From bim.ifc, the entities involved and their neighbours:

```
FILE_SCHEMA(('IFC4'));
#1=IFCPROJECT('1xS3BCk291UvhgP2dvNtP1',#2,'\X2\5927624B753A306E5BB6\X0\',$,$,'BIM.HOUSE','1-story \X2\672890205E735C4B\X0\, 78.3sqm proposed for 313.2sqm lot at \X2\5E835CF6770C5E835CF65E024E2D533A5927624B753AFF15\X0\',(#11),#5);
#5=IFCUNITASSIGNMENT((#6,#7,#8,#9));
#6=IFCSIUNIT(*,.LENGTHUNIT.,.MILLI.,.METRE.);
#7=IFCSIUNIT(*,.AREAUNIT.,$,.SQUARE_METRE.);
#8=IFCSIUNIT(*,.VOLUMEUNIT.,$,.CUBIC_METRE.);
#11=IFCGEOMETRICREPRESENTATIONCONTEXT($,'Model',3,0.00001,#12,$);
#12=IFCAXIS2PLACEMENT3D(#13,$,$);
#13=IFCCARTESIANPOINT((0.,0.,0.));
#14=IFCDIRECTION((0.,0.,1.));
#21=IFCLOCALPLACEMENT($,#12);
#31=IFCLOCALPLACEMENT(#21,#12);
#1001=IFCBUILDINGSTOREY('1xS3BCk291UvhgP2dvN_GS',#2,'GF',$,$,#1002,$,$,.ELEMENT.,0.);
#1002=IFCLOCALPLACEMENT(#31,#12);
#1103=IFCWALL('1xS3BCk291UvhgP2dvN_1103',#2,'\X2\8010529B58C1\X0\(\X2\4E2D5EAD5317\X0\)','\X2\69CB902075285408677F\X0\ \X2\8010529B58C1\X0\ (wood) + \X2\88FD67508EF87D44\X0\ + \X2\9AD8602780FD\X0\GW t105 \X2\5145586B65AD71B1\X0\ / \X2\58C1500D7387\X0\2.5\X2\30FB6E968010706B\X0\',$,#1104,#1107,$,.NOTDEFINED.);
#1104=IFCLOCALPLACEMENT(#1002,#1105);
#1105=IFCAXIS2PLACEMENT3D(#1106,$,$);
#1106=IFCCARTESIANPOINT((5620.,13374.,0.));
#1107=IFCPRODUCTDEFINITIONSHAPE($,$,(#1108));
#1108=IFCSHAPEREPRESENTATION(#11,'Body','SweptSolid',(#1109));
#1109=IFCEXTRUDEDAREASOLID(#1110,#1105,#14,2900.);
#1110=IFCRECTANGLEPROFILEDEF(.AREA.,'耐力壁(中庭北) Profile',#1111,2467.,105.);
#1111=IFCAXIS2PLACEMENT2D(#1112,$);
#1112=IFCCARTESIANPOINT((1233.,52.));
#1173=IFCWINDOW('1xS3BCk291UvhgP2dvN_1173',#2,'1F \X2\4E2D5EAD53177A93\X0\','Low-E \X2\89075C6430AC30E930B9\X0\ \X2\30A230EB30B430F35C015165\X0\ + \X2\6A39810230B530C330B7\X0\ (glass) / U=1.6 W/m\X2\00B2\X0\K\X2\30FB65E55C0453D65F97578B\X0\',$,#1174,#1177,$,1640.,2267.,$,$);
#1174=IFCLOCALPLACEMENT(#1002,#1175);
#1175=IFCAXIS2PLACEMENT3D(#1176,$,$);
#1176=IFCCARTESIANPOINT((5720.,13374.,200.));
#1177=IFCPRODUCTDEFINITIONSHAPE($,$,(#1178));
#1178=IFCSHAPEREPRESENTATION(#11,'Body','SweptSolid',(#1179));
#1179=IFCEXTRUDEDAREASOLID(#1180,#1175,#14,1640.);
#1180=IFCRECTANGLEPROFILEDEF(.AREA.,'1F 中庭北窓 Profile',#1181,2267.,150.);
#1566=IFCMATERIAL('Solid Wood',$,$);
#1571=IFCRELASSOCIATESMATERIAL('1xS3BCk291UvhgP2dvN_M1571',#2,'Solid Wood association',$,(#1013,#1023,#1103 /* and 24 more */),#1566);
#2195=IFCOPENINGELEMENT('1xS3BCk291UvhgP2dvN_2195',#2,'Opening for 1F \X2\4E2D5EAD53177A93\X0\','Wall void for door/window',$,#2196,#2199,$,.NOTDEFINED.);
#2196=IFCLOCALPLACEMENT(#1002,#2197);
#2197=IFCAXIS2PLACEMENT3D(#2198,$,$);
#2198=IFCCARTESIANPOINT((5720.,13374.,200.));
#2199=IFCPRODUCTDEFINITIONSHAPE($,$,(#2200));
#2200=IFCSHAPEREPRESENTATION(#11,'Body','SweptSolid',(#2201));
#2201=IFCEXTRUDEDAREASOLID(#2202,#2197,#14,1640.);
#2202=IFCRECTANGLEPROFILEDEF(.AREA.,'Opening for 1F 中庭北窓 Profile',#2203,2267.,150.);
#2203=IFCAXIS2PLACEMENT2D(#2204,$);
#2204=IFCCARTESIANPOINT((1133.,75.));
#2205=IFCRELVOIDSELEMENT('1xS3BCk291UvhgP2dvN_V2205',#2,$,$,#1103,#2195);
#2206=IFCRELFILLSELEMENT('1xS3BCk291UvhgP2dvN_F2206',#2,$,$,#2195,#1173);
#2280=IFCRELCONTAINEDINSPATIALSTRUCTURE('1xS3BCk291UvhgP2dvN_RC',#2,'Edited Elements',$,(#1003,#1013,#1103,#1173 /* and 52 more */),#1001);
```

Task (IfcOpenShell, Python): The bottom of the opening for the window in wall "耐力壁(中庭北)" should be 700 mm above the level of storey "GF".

```python
import numpy as np
import ifcopenshell
import ifcopenshell.api.geometry
import ifcopenshell.geom
import ifcopenshell.util.element
import ifcopenshell.util.placement
import ifcopenshell.util.shape
import ifcopenshell.util.unit

model = ifcopenshell.open("bim.ifc")
unit_scale = ifcopenshell.util.unit.calculate_unit_scale(model)

window = model.by_guid("1xS3BCk291UvhgP2dvN_1173")
opening = window.FillsVoids[0].RelatingOpeningElement
storey = ifcopenshell.util.element.get_container(window, ifc_class="IfcBuildingStorey")
level = ifcopenshell.util.placement.get_local_placement(storey.ObjectPlacement)[2, 3]

# The opening's origin need not be at the sill, so measure its lowest point.
shape = ifcopenshell.geom.create_shape(ifcopenshell.geom.settings(), opening)
bottom = ifcopenshell.util.shape.get_shape_bottom_elevation(shape, shape.geometry) / unit_scale
dz = level + 700.0 - bottom

shift = np.array([0.0, 0.0, dz])
# The window is not placed relative to its opening, so move both.
for product in (opening, window):
    matrix = ifcopenshell.util.placement.get_local_placement(product.ObjectPlacement)
    matrix[:3, 3] += shift
    ifcopenshell.api.geometry.edit_object_placement(model, product=product, matrix=matrix, is_si=False)

print(f"moved by {dz * unit_scale:+.3f} m")

model.write("bim_v2.ifc")
```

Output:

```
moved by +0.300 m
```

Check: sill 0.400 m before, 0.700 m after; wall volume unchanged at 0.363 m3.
